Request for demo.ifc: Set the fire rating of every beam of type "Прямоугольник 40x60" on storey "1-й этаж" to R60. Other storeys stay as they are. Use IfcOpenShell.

First a look at what the model holds.

```python
import ifcopenshell
import ifcopenshell.util.element

model = ifcopenshell.open("demo.ifc")
print(model.schema)
storey = next(s for s in model.by_type("IfcBuildingStorey") if s.Name == "1-й этаж")
beams = [e for e in ifcopenshell.util.element.get_decomposition(storey) if e.is_a("IfcBeam")]
seen = {}
for e in beams:
    element_type = ifcopenshell.util.element.get_type(e)
    key = (element_type.Name if element_type != e and element_type else None, ifcopenshell.util.element.get_pset(e, "Pset_BeamCommon", "FireRating"))
    seen[key] = seen.get(key, 0) + 1
for (name, value), count in sorted(seen.items(), key=str):
    print(count, "x", name, "|", value)
```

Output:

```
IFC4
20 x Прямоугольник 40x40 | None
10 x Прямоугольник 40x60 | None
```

```python
import ifcopenshell
import ifcopenshell.api.pset
import ifcopenshell.util.element

model = ifcopenshell.open("demo.ifc")

storey = next(s for s in model.by_type("IfcBuildingStorey") if s.Name == "1-й этаж")
beams = [e for e in ifcopenshell.util.element.get_decomposition(storey) if e.is_a("IfcBeam")]

count = 0
for e in beams:
    element_type = ifcopenshell.util.element.get_type(e)
    if element_type in (None, e) or element_type.Name != "Прямоугольник 40x60":
        continue
    # add_pset returns the element's existing set when there is one.
    pset = ifcopenshell.api.pset.add_pset(model, product=e, name="Pset_BeamCommon")
    ifcopenshell.api.pset.edit_pset(model, pset=pset, properties={"FireRating": "R60"})
    count += 1

print(count, "beams updated")

model.write("demo_updated.ifc")
```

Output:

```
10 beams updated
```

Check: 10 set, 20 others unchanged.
